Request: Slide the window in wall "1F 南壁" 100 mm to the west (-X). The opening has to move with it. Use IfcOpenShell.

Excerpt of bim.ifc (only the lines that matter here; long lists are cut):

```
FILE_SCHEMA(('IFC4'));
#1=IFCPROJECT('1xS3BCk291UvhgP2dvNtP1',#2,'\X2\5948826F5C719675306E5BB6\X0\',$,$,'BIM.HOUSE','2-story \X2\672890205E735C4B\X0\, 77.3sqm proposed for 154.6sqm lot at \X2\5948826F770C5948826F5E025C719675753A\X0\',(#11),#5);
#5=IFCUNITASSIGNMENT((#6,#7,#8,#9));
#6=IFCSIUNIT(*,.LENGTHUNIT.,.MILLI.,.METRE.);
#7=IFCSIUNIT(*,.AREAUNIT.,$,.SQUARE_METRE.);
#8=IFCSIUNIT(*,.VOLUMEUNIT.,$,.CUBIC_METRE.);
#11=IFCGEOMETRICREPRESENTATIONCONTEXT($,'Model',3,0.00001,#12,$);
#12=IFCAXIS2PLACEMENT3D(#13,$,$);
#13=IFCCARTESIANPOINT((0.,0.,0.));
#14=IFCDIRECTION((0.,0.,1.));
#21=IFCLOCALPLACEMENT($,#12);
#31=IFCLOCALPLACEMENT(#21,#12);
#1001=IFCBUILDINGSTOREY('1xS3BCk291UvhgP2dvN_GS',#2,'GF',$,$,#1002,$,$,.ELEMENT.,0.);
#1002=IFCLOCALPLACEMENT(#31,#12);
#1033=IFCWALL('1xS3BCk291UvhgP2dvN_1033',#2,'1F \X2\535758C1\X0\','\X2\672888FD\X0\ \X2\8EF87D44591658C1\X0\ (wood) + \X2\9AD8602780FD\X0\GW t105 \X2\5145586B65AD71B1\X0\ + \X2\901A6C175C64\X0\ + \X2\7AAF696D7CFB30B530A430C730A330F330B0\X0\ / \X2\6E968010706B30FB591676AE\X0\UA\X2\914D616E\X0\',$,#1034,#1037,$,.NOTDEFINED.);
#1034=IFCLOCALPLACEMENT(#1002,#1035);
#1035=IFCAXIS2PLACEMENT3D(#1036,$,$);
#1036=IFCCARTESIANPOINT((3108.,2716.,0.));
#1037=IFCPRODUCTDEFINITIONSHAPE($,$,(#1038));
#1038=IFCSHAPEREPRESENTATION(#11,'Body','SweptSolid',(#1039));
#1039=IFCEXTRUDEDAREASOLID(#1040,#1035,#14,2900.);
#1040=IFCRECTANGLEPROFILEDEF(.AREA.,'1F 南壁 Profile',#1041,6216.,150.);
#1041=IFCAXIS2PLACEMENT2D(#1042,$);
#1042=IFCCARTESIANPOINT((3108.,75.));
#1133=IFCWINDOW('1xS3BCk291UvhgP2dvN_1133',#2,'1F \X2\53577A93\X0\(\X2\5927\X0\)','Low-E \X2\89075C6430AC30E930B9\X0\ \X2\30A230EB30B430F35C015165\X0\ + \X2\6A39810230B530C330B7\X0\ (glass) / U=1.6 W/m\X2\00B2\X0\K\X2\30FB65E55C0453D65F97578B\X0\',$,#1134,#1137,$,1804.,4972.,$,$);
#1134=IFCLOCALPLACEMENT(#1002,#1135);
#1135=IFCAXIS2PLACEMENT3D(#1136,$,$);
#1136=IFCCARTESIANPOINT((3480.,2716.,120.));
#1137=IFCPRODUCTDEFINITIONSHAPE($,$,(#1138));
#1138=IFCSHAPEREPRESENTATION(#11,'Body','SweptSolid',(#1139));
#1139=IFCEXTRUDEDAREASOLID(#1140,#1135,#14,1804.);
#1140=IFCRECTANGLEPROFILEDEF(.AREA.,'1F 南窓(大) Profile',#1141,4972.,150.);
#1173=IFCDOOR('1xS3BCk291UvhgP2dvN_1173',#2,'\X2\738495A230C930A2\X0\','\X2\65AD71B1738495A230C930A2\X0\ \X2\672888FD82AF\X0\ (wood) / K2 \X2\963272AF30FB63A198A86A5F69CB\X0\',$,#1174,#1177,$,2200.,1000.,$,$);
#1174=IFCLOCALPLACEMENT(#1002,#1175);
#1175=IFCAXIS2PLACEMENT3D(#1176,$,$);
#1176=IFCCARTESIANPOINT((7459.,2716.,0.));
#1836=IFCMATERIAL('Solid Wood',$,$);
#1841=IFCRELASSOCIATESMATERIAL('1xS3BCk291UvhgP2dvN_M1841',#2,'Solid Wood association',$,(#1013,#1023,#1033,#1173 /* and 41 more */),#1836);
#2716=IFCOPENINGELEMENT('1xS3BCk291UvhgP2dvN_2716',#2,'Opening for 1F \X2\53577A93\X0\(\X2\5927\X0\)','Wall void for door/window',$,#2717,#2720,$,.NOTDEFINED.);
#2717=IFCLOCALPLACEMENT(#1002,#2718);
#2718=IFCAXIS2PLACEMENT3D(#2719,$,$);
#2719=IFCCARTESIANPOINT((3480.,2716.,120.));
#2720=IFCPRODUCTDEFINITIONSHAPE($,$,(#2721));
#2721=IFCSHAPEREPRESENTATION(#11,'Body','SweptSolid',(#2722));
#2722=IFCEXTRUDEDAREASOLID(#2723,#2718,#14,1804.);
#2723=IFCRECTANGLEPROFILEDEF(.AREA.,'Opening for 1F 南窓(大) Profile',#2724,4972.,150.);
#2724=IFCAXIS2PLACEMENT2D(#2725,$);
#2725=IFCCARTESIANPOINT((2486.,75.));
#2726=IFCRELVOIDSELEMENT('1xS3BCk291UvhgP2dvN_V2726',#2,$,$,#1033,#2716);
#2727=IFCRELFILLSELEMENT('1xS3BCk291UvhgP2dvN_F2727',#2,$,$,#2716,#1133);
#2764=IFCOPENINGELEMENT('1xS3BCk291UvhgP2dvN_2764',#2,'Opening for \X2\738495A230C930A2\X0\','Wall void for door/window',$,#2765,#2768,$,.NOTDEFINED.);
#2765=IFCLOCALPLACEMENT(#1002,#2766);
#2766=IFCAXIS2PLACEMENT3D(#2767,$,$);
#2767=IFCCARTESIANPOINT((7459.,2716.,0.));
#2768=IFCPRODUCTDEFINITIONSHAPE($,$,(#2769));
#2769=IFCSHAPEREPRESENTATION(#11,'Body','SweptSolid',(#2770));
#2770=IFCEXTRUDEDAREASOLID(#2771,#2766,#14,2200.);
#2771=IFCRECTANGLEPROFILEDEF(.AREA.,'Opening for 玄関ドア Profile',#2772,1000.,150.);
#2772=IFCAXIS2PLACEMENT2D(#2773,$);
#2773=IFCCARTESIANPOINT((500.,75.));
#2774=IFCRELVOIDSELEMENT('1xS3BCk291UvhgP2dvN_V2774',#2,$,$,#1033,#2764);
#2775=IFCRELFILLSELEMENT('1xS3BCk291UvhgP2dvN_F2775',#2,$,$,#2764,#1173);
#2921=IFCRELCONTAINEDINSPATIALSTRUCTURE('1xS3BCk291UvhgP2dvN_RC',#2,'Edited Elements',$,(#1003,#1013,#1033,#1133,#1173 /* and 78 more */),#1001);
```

```python
import ifcopenshell
import ifcopenshell.api.geometry
import ifcopenshell.util.placement
import ifcopenshell.util.unit

model = ifcopenshell.open("bim.ifc")
unit_scale = ifcopenshell.util.unit.calculate_unit_scale(model)

window = model.by_guid("1xS3BCk291UvhgP2dvN_1133")
opening = window.FillsVoids[0].RelatingOpeningElement
wall = opening.VoidsElements[0].RelatingBuildingElement

wall_matrix = ifcopenshell.util.placement.get_local_placement(wall.ObjectPlacement)
shift = wall_matrix[:3, 0] * -0.1 / unit_scale
before = ifcopenshell.util.placement.get_local_placement(window.ObjectPlacement)[:3, 3].copy()

# The window is not placed relative to its opening, so move both.
for product in (opening, window):
    matrix = ifcopenshell.util.placement.get_local_placement(product.ObjectPlacement)
    matrix[:3, 3] += shift
    ifcopenshell.api.geometry.edit_object_placement(model, product=product, matrix=matrix, is_si=False)

after = ifcopenshell.util.placement.get_local_placement(window.ObjectPlacement)[:3, 3]
print("window moved by", (after - before).round(3) + 0.0)

model.write("bim-out.ifc")
```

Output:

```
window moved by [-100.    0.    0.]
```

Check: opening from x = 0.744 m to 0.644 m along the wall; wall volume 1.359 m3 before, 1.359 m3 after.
